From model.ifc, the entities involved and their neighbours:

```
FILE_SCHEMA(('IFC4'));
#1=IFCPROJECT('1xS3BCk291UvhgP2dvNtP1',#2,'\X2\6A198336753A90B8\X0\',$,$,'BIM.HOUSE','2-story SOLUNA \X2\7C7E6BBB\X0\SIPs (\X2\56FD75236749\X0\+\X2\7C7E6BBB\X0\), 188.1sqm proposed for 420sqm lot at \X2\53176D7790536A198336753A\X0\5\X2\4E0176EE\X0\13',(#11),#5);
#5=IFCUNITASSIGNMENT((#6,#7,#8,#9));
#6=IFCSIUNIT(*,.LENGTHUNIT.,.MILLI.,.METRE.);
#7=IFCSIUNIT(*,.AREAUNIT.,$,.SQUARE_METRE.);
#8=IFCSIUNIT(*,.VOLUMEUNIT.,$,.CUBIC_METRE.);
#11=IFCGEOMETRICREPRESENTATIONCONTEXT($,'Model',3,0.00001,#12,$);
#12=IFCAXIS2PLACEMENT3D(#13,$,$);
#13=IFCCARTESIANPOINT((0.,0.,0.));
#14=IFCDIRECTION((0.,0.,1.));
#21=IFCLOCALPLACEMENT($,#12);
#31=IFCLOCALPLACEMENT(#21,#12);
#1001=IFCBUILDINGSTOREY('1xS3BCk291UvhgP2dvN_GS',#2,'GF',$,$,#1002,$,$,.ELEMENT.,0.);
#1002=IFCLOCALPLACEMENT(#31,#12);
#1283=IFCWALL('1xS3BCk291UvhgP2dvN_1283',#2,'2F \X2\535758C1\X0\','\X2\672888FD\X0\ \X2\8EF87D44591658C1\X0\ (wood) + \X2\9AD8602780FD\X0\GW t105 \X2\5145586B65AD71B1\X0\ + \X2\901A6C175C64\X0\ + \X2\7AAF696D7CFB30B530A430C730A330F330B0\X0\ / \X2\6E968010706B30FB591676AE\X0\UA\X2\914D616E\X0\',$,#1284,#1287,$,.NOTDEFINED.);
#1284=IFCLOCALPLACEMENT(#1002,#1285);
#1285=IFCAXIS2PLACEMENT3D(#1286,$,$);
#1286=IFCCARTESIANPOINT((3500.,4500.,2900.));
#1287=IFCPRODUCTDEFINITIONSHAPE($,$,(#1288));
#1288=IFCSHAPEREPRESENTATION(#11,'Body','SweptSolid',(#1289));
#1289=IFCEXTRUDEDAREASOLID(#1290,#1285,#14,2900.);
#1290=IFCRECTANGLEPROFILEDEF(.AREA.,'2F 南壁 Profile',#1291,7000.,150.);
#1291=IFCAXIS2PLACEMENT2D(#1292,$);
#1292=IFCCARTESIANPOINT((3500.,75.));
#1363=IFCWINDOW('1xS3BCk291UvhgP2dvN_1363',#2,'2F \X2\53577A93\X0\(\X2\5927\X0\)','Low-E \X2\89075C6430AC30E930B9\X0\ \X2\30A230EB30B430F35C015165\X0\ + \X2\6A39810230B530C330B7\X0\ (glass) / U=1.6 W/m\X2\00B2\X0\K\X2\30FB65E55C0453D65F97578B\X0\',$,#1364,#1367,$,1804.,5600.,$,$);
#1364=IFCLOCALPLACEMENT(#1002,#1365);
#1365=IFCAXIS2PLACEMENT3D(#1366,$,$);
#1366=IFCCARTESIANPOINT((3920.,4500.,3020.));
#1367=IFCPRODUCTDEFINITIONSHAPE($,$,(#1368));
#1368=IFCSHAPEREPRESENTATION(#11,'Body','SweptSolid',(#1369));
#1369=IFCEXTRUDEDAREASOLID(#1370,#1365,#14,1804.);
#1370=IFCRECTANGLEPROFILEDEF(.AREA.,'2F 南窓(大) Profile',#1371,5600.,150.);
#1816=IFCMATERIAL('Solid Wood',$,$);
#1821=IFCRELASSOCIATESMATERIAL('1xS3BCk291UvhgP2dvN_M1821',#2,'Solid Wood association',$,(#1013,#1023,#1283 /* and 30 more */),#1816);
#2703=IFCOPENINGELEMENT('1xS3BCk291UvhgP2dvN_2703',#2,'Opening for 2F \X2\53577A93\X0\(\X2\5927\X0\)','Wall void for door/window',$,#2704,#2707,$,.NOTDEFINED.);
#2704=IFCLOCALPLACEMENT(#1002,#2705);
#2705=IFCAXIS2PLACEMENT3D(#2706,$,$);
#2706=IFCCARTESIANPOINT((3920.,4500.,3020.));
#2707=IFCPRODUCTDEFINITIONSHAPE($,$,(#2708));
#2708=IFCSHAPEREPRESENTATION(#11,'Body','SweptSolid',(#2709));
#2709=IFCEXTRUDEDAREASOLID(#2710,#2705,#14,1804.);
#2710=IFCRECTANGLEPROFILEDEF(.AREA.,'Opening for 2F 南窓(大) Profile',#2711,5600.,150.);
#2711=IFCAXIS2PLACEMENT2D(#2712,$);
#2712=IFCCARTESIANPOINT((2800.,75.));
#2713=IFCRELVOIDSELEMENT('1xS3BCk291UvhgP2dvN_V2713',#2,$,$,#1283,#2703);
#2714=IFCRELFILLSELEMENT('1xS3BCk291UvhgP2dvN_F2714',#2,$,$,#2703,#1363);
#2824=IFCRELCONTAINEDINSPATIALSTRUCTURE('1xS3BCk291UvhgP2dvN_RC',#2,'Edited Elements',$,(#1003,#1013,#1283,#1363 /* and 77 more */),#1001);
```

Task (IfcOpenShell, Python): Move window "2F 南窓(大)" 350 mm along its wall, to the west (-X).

```python
import ifcopenshell
import ifcopenshell.api.geometry
import ifcopenshell.util.placement

model = ifcopenshell.open("model.ifc")

window = model.by_id(1363)
opening = window.FillsVoids[0].RelatingOpeningElement
wall = opening.VoidsElements[0].RelatingBuildingElement

wall_matrix = ifcopenshell.util.placement.get_local_placement(wall.ObjectPlacement)
shift = wall_matrix[:3, 0] * -350.0
before = ifcopenshell.util.placement.get_local_placement(window.ObjectPlacement)[:3, 3].copy()

# The window is not placed relative to its opening, so move both.
for product in (opening, window):
    matrix = ifcopenshell.util.placement.get_local_placement(product.ObjectPlacement)
    matrix[:3, 3] += shift
    ifcopenshell.api.geometry.edit_object_placement(model, product=product, matrix=matrix, is_si=False)

after = ifcopenshell.util.placement.get_local_placement(window.ObjectPlacement)[:3, 3]
print("window moved by", (after - before).round(3) + 0.0)

model.write("model_v2.ifc")
```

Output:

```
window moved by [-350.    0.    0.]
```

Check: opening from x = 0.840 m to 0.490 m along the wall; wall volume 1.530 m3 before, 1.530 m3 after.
